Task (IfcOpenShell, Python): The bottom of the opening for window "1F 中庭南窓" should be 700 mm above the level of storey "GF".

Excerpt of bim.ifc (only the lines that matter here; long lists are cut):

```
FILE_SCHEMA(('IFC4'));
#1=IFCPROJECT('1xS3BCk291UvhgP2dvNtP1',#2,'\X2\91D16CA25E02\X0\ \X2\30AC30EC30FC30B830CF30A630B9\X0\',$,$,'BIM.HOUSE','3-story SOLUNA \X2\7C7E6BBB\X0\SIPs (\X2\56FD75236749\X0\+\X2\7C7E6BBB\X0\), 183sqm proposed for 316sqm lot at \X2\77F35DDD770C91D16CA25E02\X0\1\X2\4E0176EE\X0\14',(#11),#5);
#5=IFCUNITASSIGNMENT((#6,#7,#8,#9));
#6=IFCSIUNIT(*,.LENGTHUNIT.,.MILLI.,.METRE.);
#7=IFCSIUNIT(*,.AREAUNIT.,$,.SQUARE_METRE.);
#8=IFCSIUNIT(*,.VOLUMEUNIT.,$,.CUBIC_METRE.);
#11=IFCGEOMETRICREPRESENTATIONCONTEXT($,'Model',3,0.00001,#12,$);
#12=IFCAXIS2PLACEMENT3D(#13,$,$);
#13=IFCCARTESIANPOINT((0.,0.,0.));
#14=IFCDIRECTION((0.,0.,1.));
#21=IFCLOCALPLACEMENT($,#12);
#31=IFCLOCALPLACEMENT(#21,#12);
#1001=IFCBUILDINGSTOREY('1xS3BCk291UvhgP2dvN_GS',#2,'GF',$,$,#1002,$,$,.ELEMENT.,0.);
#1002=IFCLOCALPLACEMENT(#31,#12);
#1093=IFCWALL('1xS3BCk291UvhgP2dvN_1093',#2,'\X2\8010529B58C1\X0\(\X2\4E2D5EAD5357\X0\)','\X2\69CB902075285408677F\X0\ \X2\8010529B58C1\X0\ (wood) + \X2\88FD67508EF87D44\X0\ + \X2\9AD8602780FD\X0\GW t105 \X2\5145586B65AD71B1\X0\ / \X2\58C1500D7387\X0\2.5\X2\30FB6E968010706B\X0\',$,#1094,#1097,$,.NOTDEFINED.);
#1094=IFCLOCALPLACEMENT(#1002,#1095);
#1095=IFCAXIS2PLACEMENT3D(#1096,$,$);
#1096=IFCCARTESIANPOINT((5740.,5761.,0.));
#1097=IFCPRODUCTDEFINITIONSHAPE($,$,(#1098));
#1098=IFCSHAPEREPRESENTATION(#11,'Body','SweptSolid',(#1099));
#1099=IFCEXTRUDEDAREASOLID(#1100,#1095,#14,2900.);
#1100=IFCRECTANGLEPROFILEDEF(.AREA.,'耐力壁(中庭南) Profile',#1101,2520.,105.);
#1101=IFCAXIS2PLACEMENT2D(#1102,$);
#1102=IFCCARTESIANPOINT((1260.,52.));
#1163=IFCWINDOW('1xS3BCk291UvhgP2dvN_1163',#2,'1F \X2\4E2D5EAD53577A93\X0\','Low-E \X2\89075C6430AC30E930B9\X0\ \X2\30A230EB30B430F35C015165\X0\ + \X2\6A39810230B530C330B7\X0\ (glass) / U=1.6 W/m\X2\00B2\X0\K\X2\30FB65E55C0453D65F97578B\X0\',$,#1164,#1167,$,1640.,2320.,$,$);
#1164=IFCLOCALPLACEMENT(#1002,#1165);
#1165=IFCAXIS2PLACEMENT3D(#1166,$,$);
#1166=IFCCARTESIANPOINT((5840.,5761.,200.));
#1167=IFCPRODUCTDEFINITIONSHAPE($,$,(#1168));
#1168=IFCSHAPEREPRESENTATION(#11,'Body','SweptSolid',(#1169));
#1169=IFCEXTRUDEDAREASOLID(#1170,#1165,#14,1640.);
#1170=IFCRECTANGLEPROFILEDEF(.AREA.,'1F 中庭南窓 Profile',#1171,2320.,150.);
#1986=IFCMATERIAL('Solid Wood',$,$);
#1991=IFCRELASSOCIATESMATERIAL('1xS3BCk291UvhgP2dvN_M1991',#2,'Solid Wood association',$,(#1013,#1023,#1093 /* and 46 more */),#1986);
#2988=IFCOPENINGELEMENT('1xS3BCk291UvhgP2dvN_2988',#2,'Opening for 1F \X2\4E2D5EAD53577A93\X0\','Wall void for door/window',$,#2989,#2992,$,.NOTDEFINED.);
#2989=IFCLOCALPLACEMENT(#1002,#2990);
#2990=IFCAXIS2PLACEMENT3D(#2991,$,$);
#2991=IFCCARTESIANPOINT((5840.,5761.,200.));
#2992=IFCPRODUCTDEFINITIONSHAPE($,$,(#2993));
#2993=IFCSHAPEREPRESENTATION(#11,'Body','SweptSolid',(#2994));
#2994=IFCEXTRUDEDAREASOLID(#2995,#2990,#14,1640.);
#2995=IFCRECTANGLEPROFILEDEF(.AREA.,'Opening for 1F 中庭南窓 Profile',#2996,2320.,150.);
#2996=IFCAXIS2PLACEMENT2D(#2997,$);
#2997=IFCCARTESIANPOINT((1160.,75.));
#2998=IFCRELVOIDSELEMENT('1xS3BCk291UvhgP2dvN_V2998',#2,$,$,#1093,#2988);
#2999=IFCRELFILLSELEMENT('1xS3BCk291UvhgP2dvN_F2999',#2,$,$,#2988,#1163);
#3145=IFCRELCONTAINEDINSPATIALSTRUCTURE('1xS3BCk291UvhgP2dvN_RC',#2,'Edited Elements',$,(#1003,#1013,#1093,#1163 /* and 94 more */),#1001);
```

```python
import numpy as np
import ifcopenshell
import ifcopenshell.api.geometry
import ifcopenshell.geom
import ifcopenshell.util.element
import ifcopenshell.util.placement
import ifcopenshell.util.shape
import ifcopenshell.util.unit

model = ifcopenshell.open("bim.ifc")
unit_scale = ifcopenshell.util.unit.calculate_unit_scale(model)

window = model.by_guid("1xS3BCk291UvhgP2dvN_1163")
opening = window.FillsVoids[0].RelatingOpeningElement
storey = ifcopenshell.util.element.get_container(window, ifc_class="IfcBuildingStorey")
level = ifcopenshell.util.placement.get_local_placement(storey.ObjectPlacement)[2, 3]

# The opening's origin need not be at the sill, so measure its lowest point.
shape = ifcopenshell.geom.create_shape(ifcopenshell.geom.settings(), opening)
bottom = ifcopenshell.util.shape.get_shape_bottom_elevation(shape, shape.geometry) / unit_scale
dz = level + 700.0 - bottom

shift = np.array([0.0, 0.0, dz])
# The window is not placed relative to its opening, so move both.
for product in (opening, window):
    matrix = ifcopenshell.util.placement.get_local_placement(product.ObjectPlacement)
    matrix[:3, 3] += shift
    ifcopenshell.api.geometry.edit_object_placement(model, product=product, matrix=matrix, is_si=False)

print(f"moved by {dz * unit_scale:+.3f} m")

model.write("bim_edited.ifc")
```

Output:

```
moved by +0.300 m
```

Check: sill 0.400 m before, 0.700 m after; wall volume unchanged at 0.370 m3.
